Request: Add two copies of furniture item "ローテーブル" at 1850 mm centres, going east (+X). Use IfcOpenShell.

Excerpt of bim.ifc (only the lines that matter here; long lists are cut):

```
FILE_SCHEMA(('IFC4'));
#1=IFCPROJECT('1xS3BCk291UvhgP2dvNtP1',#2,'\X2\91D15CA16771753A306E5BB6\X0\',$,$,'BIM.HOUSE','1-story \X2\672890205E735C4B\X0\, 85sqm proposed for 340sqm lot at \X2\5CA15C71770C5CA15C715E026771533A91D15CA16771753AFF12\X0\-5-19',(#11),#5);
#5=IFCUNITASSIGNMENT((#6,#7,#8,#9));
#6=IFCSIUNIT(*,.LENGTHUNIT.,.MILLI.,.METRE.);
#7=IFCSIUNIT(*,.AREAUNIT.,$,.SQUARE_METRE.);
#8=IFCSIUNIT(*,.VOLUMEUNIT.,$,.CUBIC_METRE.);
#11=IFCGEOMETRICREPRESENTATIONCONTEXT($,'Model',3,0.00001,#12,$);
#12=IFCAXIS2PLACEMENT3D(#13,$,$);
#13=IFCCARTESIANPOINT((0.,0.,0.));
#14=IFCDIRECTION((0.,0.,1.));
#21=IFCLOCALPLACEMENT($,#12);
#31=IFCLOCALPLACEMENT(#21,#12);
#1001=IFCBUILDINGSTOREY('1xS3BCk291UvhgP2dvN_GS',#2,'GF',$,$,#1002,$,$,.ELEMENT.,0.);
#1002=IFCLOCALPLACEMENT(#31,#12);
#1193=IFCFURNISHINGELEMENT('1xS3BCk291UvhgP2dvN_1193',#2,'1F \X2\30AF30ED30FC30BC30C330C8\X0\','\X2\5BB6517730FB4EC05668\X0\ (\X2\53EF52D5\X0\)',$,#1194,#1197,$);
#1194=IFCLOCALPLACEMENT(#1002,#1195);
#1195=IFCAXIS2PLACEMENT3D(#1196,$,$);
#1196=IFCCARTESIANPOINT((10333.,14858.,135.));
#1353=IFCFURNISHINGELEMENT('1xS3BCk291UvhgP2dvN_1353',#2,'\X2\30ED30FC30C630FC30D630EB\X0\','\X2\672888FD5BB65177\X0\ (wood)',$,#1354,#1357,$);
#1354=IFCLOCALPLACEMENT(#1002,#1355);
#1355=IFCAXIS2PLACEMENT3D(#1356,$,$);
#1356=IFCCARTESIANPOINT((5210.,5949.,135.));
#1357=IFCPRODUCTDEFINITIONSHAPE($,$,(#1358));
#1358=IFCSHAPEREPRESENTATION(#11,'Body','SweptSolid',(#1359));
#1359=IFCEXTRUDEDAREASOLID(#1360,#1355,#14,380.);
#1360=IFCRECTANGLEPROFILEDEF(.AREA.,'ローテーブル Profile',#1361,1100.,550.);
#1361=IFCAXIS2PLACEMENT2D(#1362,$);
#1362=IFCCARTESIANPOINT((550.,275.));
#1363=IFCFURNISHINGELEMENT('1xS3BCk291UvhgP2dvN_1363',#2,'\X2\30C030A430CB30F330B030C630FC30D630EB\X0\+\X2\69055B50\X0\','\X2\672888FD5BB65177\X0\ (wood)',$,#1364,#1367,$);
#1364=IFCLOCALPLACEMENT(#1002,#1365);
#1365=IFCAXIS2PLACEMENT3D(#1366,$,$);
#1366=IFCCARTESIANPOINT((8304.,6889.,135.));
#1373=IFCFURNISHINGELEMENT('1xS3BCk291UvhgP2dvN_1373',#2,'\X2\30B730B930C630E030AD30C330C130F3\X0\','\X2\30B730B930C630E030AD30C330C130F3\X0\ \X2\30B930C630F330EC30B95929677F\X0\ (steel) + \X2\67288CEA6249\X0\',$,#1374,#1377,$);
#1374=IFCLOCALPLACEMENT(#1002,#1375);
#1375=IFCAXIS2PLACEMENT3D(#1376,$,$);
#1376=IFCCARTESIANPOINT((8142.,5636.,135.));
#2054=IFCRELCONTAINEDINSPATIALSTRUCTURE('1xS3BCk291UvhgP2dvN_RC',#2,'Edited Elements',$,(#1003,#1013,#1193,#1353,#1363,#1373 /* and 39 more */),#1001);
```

```python
import numpy as np
import ifcopenshell
import ifcopenshell.api.geometry
import ifcopenshell.api.root
import ifcopenshell.util.element
import ifcopenshell.util.placement
import ifcopenshell.util.unit

model = ifcopenshell.open("bim.ifc")
unit_scale = ifcopenshell.util.unit.calculate_unit_scale(model)


def reuse_history(source, copy):
    """copy_class also copies each property set's owner history, people and application; keep the originals."""
    for rel in copy.IsDefinedBy:
        if rel.is_a("IfcRelDefinesByProperties") and (history := rel.RelatingPropertyDefinition.OwnerHistory):
            rel.RelatingPropertyDefinition.OwnerHistory = source.OwnerHistory
            ifcopenshell.util.element.remove_deep2(model, history)


source = model.by_guid("1xS3BCk291UvhgP2dvN_1353")
base = ifcopenshell.util.placement.get_local_placement(source.ObjectPlacement)
step = np.array([1.0, 0.0, 0.0]) * 1.85 / unit_scale

for i in range(1, 3):
    copy = ifcopenshell.api.root.copy_class(model, product=source)
    copy.Representation = ifcopenshell.util.element.copy_deep(
        model, source.Representation, exclude=["IfcGeometricRepresentationContext", "IfcRepresentationMap"]
    )
    reuse_history(source, copy)
    matrix = base.copy()
    matrix[:3, 3] += i * step
    print("added at", matrix[:3, 3].round(3) + 0.0)
    ifcopenshell.api.geometry.edit_object_placement(model, product=copy, matrix=matrix, is_si=False)

model.write("bim-out.ifc")
```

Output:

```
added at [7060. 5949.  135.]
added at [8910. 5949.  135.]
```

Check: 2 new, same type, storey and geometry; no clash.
